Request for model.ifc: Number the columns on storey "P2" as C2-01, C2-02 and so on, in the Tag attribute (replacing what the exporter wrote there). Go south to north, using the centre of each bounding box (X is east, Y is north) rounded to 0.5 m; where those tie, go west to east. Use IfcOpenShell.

First a look at what the model holds.

```python
import ifcopenshell
import ifcopenshell.util.element
import ifcopenshell.util.placement

model = ifcopenshell.open("model.ifc")
print(model.schema)
storey = next(s for s in model.by_type("IfcBuildingStorey") if s.Name == "P2")
columns = [e for e in ifcopenshell.util.element.get_decomposition(storey) if e.is_a("IfcColumn")]
for e in sorted(columns, key=lambda e: e.id()):
    origin = ifcopenshell.util.placement.get_local_placement(e.ObjectPlacement)[:3, 3]
    print(e.id(), e.Tag, e.Name, origin.round(2) + 0.0, sep=" | ")
```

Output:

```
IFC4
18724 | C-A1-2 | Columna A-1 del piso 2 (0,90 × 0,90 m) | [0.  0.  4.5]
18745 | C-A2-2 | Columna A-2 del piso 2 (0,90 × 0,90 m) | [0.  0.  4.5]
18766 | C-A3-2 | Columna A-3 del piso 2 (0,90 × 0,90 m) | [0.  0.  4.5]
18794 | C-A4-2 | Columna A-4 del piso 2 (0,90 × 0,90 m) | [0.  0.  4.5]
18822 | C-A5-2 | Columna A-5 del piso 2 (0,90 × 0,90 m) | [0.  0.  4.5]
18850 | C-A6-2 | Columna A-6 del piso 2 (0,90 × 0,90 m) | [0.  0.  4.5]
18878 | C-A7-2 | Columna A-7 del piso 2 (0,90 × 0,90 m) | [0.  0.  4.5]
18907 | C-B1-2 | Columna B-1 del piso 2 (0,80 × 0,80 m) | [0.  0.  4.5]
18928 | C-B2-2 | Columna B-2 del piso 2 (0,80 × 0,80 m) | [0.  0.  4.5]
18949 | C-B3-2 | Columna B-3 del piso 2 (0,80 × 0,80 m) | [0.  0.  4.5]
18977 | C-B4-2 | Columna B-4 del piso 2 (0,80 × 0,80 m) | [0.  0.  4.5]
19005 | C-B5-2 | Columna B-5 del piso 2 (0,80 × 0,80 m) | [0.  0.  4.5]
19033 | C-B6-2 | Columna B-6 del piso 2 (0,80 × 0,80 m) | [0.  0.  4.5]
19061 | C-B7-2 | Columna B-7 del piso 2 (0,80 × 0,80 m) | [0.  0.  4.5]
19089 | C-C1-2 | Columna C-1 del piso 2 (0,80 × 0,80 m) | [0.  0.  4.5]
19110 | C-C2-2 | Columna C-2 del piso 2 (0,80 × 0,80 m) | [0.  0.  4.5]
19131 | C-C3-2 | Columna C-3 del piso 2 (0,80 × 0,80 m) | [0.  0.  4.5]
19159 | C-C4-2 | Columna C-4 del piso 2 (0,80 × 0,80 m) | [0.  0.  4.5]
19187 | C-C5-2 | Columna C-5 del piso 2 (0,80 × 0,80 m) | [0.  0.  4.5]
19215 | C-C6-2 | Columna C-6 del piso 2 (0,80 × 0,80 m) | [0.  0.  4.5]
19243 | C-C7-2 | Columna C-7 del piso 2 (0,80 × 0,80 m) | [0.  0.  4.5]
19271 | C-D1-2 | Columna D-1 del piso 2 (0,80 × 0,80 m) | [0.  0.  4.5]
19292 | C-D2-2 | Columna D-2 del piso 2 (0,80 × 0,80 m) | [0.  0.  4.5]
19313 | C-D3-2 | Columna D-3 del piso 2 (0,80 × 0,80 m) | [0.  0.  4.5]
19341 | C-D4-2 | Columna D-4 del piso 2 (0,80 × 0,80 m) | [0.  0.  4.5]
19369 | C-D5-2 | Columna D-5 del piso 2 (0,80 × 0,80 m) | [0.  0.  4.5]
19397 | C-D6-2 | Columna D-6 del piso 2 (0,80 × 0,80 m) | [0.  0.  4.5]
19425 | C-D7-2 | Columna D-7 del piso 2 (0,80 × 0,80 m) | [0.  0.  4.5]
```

```python
import ifcopenshell
import ifcopenshell.geom
import ifcopenshell.util.element
import ifcopenshell.util.shape

model = ifcopenshell.open("model.ifc")
settings = ifcopenshell.geom.settings()
settings.set("use-world-coords", True)


def centre(element):
    shape = ifcopenshell.geom.create_shape(settings, element)
    return ifcopenshell.util.shape.get_bbox_centroid(shape.geometry)


storey = next(s for s in model.by_type("IfcBuildingStorey") if s.Name == "P2")
columns = [e for e in ifcopenshell.util.element.get_decomposition(storey) if e.is_a("IfcColumn")]

# Insertion points can sit at a corner or the storey origin, so sort by the geometry (in metres).
centres = {e: centre(e) for e in columns}
columns.sort(key=lambda e: (round(centres[e][1] / 0.5), centres[e][0]))

for i, e in enumerate(columns, start=1):
    number = f"C2-{i:02d}"
    e.Tag = number
    print(e.id(), number)

model.write("model_v2.ifc")
```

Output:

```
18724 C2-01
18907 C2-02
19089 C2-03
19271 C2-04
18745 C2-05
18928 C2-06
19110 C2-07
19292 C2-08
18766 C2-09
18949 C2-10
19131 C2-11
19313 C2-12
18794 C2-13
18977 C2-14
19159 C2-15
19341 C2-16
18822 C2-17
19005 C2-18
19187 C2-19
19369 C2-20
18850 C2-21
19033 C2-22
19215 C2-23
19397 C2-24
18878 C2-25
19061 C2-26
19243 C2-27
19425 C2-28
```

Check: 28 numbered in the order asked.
